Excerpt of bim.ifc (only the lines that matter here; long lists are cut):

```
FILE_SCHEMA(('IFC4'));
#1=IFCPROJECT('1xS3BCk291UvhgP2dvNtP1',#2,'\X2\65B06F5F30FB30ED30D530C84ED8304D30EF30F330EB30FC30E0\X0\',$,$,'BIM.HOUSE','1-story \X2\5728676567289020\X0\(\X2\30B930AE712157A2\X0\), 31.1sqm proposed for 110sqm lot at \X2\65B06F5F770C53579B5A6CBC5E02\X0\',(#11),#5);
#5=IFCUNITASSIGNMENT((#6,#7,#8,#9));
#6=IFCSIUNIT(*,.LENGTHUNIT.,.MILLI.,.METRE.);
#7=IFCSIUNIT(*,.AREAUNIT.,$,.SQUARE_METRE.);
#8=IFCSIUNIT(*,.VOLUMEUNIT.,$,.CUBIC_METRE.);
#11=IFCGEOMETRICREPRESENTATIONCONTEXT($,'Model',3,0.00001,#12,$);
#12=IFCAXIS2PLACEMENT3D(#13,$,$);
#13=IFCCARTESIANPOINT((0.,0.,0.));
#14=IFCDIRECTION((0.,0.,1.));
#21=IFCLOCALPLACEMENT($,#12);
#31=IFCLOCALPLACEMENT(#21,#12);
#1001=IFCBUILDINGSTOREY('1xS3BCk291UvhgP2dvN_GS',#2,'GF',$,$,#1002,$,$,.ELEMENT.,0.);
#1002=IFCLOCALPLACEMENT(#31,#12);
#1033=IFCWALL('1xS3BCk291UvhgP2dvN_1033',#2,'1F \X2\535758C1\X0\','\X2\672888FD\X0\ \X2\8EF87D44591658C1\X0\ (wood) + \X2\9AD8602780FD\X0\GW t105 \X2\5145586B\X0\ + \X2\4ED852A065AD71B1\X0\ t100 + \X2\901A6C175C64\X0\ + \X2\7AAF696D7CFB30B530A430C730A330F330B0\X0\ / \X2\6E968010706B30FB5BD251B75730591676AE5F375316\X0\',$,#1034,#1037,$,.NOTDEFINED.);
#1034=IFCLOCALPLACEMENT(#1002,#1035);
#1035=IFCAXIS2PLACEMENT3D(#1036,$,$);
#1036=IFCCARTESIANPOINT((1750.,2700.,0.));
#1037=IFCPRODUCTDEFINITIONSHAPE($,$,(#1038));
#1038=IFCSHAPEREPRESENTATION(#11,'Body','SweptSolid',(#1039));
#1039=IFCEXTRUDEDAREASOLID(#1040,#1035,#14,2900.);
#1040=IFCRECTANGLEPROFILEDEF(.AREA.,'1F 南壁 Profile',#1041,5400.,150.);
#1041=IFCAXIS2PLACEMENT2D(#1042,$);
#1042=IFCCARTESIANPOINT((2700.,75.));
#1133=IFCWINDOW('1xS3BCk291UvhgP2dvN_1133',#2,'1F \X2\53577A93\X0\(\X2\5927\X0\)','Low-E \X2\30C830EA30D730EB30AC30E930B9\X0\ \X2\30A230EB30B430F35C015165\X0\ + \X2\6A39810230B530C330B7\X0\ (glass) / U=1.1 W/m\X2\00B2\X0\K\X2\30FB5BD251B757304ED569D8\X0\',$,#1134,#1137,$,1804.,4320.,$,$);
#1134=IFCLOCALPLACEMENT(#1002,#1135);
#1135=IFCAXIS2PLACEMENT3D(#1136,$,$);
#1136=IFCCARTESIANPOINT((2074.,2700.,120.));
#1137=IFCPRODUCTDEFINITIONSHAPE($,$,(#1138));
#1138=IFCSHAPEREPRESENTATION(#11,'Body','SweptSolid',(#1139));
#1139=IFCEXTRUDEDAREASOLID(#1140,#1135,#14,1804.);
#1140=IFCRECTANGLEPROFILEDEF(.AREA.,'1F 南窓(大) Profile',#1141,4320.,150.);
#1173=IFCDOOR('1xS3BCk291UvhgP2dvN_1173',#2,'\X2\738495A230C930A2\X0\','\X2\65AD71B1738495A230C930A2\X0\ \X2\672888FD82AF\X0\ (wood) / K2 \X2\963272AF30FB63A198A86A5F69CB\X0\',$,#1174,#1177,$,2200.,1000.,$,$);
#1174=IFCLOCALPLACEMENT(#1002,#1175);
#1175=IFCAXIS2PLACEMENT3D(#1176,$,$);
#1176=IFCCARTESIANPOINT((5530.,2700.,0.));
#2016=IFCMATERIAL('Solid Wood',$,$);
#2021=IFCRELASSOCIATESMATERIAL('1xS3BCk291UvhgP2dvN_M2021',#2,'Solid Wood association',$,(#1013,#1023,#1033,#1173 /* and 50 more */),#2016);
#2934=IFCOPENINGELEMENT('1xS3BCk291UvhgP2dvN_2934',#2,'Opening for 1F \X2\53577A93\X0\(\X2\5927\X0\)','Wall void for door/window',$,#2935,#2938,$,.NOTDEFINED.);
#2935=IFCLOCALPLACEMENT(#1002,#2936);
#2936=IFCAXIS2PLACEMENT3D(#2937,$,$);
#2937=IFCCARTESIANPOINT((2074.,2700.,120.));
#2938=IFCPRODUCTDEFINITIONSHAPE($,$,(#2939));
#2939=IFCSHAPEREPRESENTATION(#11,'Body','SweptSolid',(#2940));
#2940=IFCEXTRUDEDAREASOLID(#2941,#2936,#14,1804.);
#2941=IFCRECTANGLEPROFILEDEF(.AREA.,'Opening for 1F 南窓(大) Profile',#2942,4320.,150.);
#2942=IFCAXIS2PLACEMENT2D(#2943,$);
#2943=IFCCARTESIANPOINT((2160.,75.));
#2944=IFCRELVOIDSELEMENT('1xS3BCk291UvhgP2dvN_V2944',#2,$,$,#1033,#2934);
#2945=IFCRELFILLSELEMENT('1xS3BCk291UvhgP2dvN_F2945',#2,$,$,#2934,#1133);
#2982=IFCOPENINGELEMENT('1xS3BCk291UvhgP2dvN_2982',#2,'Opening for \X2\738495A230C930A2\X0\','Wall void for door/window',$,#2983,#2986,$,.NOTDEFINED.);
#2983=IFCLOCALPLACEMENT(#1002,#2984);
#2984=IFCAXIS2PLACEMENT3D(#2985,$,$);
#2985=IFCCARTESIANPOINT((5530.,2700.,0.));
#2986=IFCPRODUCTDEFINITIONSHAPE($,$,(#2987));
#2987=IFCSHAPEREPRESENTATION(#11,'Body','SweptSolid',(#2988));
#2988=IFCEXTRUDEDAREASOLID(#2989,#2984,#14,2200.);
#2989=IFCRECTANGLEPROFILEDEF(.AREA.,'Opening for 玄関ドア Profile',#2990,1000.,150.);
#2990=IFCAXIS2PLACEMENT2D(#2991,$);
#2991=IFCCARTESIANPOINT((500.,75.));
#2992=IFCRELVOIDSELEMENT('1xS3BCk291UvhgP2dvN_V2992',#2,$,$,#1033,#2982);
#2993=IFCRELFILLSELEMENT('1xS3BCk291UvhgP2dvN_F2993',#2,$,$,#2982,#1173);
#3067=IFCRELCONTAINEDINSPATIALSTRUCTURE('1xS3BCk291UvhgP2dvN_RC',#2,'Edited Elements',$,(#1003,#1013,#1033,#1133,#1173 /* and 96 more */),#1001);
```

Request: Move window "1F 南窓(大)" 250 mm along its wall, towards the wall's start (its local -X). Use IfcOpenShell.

```python
import ifcopenshell
import ifcopenshell.api.geometry
import ifcopenshell.util.placement
import ifcopenshell.util.unit

model = ifcopenshell.open("bim.ifc")
unit_scale = ifcopenshell.util.unit.calculate_unit_scale(model)

window = model.by_guid("1xS3BCk291UvhgP2dvN_1133")
opening = window.FillsVoids[0].RelatingOpeningElement
wall = opening.VoidsElements[0].RelatingBuildingElement

wall_matrix = ifcopenshell.util.placement.get_local_placement(wall.ObjectPlacement)
shift = wall_matrix[:3, 0] * -0.25 / unit_scale
before = ifcopenshell.util.placement.get_local_placement(window.ObjectPlacement)[:3, 3].copy()

# The window is not placed relative to its opening, so move both.
for product in (opening, window):
    matrix = ifcopenshell.util.placement.get_local_placement(product.ObjectPlacement)
    matrix[:3, 3] += shift
    ifcopenshell.api.geometry.edit_object_placement(model, product=product, matrix=matrix, is_si=False)

after = ifcopenshell.util.placement.get_local_placement(window.ObjectPlacement)[:3, 3]
print("window moved by", (after - before).round(3) + 0.0)

model.write("bim_rev.ifc")
```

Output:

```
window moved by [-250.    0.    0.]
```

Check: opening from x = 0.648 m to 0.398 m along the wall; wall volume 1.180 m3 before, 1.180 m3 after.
